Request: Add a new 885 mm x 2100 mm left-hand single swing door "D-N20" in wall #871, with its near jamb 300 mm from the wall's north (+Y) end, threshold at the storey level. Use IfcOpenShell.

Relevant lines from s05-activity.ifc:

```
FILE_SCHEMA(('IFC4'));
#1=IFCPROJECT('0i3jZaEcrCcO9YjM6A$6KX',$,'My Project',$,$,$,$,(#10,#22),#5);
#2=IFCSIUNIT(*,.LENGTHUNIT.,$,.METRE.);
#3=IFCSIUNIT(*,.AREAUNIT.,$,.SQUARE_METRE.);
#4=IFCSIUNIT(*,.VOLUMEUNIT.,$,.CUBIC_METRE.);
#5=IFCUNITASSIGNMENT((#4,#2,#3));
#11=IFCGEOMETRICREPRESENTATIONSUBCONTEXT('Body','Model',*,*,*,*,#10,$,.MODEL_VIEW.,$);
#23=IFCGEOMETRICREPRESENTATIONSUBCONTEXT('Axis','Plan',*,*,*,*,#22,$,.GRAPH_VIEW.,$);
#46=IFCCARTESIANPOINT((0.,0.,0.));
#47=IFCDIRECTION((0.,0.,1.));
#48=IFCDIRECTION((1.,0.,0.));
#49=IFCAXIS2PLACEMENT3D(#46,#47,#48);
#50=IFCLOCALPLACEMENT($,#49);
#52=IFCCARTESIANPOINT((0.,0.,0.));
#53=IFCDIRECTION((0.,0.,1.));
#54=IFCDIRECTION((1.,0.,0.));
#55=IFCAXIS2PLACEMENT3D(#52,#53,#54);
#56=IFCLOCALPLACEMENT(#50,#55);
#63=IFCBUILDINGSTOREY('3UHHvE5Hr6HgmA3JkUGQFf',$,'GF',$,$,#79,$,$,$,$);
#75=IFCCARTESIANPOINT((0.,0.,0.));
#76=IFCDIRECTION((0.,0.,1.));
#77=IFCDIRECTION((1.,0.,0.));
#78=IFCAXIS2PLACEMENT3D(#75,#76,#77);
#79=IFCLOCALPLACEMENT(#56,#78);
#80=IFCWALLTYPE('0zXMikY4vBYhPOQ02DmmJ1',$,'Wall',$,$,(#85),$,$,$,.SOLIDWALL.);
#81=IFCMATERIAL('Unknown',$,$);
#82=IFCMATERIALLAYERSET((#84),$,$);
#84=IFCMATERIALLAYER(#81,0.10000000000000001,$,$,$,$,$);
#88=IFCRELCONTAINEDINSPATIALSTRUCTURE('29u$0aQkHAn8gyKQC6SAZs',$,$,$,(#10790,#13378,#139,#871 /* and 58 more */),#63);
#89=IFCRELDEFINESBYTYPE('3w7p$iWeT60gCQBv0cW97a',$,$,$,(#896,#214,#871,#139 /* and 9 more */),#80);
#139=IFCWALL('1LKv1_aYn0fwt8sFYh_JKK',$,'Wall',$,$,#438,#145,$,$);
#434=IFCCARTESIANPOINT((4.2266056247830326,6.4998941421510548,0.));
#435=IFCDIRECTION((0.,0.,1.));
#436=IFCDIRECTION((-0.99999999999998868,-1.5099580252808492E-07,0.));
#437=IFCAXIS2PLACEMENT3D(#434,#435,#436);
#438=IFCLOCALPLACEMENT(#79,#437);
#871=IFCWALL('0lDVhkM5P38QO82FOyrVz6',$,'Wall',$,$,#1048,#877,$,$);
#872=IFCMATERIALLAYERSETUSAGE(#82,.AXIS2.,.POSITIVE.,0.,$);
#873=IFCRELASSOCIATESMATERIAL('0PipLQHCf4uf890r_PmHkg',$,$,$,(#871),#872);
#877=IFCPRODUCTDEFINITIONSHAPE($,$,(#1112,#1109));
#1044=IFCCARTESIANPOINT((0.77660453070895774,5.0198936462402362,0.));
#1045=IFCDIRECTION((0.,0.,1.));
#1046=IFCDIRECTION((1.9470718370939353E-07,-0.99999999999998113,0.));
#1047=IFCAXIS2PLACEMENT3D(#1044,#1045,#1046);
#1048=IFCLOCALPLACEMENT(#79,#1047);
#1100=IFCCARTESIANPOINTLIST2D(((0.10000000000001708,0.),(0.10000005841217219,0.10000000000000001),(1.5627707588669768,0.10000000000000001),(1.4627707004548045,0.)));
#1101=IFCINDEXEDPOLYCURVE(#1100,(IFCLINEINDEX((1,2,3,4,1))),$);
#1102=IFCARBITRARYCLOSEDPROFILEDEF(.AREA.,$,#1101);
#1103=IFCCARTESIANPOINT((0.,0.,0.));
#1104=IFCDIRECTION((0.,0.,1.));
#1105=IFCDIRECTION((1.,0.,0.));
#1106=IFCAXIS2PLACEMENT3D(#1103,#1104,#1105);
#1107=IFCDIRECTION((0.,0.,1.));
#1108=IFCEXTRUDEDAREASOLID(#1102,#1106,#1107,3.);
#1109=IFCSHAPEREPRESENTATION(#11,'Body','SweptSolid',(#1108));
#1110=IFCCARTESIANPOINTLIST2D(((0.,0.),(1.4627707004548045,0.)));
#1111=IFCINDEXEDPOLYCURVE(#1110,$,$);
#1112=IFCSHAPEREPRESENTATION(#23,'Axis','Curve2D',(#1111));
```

```python
import numpy as np
import ifcopenshell
import ifcopenshell.api.feature
import ifcopenshell.api.geometry
import ifcopenshell.api.root
import ifcopenshell.api.spatial
import ifcopenshell.geom
import ifcopenshell.util.element
import ifcopenshell.util.placement
import ifcopenshell.util.representation
import ifcopenshell.util.shape
import ifcopenshell.util.unit

model = ifcopenshell.open("s05-activity.ifc")
unit_scale = ifcopenshell.util.unit.calculate_unit_scale(model)
settings = ifcopenshell.geom.settings()


def volume(element):
    """Net volume in cubic metres, openings subtracted."""
    shape = ifcopenshell.geom.create_shape(settings, element)
    return ifcopenshell.util.shape.get_volume(shape.geometry)


wall = model.by_id(871)
storey = ifcopenshell.util.element.get_container(wall, ifc_class="IfcBuildingStorey")
context = ifcopenshell.util.representation.get_context(model, "Model", "Body", "MODEL_VIEW")
before = volume(wall)

width, height, from_end, sill = 0.885, 2.1, 0.3, 0.0  # metres

# The wall runs along its own X axis, and the end named is its -X end.
wall_shape = ifcopenshell.geom.create_shape(settings, wall)
x, y, z = ifcopenshell.util.shape.get_vertices(wall_shape.geometry).T
start = x.min() + from_end
face, thickness = float(y.min()), float(y.max() - y.min())
wall_matrix = ifcopenshell.util.placement.get_local_placement(wall.ObjectPlacement)
level = ifcopenshell.util.placement.get_local_placement(storey.ObjectPlacement)[2, 3]


def in_wall(x, y):
    """Placement at x, y metres in the wall's axes, at sill height."""
    matrix = wall_matrix.copy()
    matrix[:, 3] = wall_matrix @ np.array([x / unit_scale, y / unit_scale, 0.0, 1.0])
    matrix[2, 3] = level + sill / unit_scale
    return matrix


# Opening: a box that overshoots both wall faces by 50 mm.
opening = ifcopenshell.api.root.create_entity(model, ifc_class="IfcOpeningElement", predefined_type="OPENING")
box = ifcopenshell.api.geometry.add_wall_representation(
    model, context=context, length=width, height=height, thickness=thickness + 0.1
)
ifcopenshell.api.geometry.assign_representation(model, product=opening, representation=box)
ifcopenshell.api.geometry.edit_object_placement(model, product=opening, matrix=in_wall(start, face - 0.05), is_si=False)
ifcopenshell.api.feature.add_feature(model, feature=opening, element=wall)

door = ifcopenshell.api.root.create_entity(model, ifc_class="IfcDoor", name="D-N20", predefined_type="DOOR")
door.OverallWidth, door.OverallHeight = width / unit_scale, height / unit_scale
door.OperationType = "SINGLE_SWING_LEFT"
body = ifcopenshell.api.geometry.add_door_representation(
    model,
    context=context,
    overall_width=door.OverallWidth,
    overall_height=door.OverallHeight,
    operation_type="SINGLE_SWING_LEFT",
    lining_properties={"LiningDepth": thickness / unit_scale, "ThresholdDepth": thickness / unit_scale},
)
ifcopenshell.api.geometry.assign_representation(model, product=door, representation=body)
ifcopenshell.api.spatial.assign_container(model, products=[door], relating_structure=storey)
ifcopenshell.api.feature.add_filling(model, opening=opening, element=door)

# The lining spans the wall, so the door starts at the wall face.
ifcopenshell.api.geometry.edit_object_placement(model, product=door, matrix=in_wall(start, face), is_si=False)

after = volume(wall)

print(f"wall volume {before:.3f} -> {after:.3f} m3")

model.write("s05-activity_edited.ifc")
```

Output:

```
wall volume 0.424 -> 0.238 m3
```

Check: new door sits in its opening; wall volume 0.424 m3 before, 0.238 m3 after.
